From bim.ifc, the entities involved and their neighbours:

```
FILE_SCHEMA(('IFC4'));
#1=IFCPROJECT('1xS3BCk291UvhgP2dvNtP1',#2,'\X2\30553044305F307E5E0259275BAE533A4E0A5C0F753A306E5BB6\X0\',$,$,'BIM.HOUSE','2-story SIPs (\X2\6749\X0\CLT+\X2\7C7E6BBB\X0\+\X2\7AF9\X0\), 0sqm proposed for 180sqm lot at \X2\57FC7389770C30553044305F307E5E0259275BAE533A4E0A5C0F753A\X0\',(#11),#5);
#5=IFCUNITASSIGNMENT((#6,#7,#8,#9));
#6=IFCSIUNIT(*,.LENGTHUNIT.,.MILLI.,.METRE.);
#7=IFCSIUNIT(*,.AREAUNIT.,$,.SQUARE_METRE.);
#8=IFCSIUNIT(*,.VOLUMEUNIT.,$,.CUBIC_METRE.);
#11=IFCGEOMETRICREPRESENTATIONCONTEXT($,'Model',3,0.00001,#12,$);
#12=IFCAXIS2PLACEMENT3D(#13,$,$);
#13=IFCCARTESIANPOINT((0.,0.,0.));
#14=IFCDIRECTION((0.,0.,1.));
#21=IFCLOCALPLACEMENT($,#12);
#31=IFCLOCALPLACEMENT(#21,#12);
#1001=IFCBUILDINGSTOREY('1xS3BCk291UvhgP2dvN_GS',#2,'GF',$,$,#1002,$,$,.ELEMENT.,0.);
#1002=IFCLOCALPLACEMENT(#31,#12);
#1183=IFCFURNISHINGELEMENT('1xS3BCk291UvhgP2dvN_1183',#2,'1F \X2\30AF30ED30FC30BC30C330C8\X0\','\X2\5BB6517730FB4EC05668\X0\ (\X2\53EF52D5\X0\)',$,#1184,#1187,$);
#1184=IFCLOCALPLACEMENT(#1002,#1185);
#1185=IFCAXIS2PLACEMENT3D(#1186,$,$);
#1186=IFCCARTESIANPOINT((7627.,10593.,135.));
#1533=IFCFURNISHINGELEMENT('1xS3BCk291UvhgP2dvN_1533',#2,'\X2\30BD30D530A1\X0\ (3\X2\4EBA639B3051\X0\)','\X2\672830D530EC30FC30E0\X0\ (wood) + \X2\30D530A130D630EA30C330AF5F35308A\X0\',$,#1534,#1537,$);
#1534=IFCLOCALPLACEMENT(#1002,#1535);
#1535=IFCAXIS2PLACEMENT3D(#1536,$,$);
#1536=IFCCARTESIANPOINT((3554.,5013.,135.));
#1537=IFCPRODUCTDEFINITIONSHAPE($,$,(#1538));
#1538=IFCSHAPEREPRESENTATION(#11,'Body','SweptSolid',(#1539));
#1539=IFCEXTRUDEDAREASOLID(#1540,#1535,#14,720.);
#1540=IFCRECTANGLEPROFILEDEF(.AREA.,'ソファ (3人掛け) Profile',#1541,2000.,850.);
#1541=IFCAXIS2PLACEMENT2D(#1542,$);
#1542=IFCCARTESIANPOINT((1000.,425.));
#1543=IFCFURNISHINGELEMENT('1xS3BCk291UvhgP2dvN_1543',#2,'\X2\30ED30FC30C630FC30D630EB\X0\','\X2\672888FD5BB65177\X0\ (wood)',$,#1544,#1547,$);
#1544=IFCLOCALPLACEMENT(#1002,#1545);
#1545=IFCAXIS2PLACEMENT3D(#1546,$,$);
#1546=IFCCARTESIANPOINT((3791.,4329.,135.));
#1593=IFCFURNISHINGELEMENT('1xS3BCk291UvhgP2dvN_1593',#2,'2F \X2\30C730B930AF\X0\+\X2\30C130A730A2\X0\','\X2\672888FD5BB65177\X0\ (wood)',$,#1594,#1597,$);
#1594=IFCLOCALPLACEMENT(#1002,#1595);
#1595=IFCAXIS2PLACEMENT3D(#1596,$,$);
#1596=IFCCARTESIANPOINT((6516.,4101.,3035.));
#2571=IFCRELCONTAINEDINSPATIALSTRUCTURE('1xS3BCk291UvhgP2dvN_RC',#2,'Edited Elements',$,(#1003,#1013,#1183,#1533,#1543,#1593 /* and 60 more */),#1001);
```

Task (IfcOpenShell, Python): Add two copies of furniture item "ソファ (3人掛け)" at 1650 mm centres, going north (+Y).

```python
import numpy as np
import ifcopenshell
import ifcopenshell.api.geometry
import ifcopenshell.api.root
import ifcopenshell.util.element
import ifcopenshell.util.placement

model = ifcopenshell.open("bim.ifc")


def reuse_history(source, copy):
    """copy_class also copies each property set's owner history, people and application; keep the originals."""
    for rel in copy.IsDefinedBy:
        if rel.is_a("IfcRelDefinesByProperties") and (history := rel.RelatingPropertyDefinition.OwnerHistory):
            rel.RelatingPropertyDefinition.OwnerHistory = source.OwnerHistory
            ifcopenshell.util.element.remove_deep2(model, history)


source = model.by_guid("1xS3BCk291UvhgP2dvN_1533")
base = ifcopenshell.util.placement.get_local_placement(source.ObjectPlacement)
step = np.array([0.0, 1.0, 0.0]) * 1650.0

for i in range(1, 3):
    copy = ifcopenshell.api.root.copy_class(model, product=source)
    copy.Representation = ifcopenshell.util.element.copy_deep(
        model, source.Representation, exclude=["IfcGeometricRepresentationContext", "IfcRepresentationMap"]
    )
    reuse_history(source, copy)
    matrix = base.copy()
    matrix[:3, 3] += i * step
    print("added at", matrix[:3, 3].round(3) + 0.0)
    ifcopenshell.api.geometry.edit_object_placement(model, product=copy, matrix=matrix, is_si=False)

model.write("bim_v2.ifc")
```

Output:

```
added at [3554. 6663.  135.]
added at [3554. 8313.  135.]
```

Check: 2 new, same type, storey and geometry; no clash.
